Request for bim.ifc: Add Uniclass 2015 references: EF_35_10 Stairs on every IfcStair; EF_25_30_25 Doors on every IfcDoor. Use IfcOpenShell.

First a look at what the model holds.

```python
import ifcopenshell

model = ifcopenshell.open("bim.ifc")
print(model.schema)
print("classifications:", [c.Name for c in model.by_type("IfcClassification")])
for ifc_class in ("IfcDoor", "IfcRoof", "IfcStair", "IfcWall", "IfcWindow"):
    print(ifc_class, len(model.by_type(ifc_class)))
```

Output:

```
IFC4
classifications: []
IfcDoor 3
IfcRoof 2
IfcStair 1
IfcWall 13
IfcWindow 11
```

```python
import ifcopenshell
import ifcopenshell.api.classification

model = ifcopenshell.open("bim.ifc")

system = ifcopenshell.api.classification.add_classification(model, classification="Uniclass 2015")

codes = {
    "IfcStair": ("EF_35_10", "Stairs"),
    "IfcDoor": ("EF_25_30_25", "Doors"),
}
for ifc_class, (code, name) in codes.items():
    products = model.by_type(ifc_class)
    ifcopenshell.api.classification.add_reference(
        model, products=products, classification=system, identification=code, name=name
    )
    print(code, len(products))

model.write("bim-out.ifc")
```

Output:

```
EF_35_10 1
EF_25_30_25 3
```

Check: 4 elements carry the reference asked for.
